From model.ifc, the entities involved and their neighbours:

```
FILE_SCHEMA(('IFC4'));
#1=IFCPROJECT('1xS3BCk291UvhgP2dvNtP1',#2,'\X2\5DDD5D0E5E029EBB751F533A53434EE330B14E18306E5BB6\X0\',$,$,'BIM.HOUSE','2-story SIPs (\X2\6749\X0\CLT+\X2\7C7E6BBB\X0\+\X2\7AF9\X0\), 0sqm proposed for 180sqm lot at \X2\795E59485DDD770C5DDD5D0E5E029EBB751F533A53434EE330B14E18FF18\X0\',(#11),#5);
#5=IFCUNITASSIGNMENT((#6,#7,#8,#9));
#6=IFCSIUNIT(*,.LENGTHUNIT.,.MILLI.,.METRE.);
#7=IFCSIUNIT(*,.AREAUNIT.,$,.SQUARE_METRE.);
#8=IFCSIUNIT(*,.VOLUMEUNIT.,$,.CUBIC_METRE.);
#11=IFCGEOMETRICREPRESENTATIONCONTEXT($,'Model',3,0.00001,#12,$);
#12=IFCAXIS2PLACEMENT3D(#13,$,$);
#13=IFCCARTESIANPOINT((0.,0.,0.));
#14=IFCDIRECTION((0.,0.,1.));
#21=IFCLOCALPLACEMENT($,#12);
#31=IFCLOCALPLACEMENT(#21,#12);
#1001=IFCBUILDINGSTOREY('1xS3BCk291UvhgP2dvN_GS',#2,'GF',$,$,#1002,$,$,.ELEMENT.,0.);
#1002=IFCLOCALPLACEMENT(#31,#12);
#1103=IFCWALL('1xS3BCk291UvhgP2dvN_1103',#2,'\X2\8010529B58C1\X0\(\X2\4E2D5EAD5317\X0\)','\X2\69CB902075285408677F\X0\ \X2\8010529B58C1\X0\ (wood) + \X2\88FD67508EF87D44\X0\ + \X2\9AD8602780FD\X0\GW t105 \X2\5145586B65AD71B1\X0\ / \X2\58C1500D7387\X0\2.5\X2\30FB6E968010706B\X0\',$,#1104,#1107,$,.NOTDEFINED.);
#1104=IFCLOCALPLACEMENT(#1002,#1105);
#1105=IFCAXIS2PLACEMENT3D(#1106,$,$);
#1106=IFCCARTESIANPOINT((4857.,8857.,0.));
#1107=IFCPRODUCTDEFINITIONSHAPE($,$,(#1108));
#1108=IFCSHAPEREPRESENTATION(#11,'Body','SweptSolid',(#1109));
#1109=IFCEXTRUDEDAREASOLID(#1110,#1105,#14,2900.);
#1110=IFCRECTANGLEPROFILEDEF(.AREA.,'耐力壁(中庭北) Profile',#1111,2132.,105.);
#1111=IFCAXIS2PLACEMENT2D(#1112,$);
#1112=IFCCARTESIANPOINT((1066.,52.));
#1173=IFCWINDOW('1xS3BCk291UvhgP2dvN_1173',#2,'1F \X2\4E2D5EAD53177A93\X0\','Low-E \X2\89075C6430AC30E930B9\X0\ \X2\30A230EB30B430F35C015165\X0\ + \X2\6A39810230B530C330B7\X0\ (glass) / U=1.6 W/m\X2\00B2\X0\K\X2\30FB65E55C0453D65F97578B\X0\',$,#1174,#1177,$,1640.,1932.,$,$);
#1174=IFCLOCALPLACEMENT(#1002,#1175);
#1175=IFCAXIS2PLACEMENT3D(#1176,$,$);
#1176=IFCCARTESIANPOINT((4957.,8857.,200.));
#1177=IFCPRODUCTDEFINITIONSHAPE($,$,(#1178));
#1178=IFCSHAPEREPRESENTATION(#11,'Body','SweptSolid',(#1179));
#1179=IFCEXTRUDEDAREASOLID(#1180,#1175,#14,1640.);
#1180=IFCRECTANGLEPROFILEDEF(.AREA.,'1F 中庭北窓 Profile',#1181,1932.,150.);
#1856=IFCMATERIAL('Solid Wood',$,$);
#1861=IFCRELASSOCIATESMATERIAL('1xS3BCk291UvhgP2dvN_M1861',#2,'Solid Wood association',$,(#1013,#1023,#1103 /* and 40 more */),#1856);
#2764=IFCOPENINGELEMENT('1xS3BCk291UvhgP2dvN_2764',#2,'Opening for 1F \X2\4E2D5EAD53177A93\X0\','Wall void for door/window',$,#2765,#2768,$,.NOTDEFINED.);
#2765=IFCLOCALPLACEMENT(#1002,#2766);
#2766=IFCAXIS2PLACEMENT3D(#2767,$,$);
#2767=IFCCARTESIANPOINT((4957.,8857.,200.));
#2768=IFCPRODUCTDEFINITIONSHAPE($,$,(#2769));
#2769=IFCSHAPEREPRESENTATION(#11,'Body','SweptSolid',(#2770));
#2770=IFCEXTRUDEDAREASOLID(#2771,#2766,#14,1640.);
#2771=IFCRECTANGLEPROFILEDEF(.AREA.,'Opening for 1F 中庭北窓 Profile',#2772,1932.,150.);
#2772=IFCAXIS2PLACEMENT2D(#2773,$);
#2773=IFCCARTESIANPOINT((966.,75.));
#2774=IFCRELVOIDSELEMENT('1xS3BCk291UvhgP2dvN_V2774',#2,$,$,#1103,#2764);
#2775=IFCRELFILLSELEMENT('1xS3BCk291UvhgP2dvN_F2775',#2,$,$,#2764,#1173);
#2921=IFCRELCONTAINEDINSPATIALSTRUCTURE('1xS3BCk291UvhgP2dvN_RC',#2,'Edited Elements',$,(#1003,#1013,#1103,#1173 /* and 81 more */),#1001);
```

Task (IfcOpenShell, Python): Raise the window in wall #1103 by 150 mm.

```python
import numpy as np
import ifcopenshell
import ifcopenshell.api.geometry
import ifcopenshell.util.placement
import ifcopenshell.util.unit

model = ifcopenshell.open("model.ifc")
unit_scale = ifcopenshell.util.unit.calculate_unit_scale(model)

window = model.by_id(1173)
opening = window.FillsVoids[0].RelatingOpeningElement
dz = 150.0

shift = np.array([0.0, 0.0, dz])
# The window is not placed relative to its opening, so move both.
for product in (opening, window):
    matrix = ifcopenshell.util.placement.get_local_placement(product.ObjectPlacement)
    matrix[:3, 3] += shift
    ifcopenshell.api.geometry.edit_object_placement(model, product=product, matrix=matrix, is_si=False)

print(f"moved by {dz * unit_scale:+.3f} m")

model.write("model_updated.ifc")
```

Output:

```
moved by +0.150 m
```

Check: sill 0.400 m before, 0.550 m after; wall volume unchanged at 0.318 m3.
